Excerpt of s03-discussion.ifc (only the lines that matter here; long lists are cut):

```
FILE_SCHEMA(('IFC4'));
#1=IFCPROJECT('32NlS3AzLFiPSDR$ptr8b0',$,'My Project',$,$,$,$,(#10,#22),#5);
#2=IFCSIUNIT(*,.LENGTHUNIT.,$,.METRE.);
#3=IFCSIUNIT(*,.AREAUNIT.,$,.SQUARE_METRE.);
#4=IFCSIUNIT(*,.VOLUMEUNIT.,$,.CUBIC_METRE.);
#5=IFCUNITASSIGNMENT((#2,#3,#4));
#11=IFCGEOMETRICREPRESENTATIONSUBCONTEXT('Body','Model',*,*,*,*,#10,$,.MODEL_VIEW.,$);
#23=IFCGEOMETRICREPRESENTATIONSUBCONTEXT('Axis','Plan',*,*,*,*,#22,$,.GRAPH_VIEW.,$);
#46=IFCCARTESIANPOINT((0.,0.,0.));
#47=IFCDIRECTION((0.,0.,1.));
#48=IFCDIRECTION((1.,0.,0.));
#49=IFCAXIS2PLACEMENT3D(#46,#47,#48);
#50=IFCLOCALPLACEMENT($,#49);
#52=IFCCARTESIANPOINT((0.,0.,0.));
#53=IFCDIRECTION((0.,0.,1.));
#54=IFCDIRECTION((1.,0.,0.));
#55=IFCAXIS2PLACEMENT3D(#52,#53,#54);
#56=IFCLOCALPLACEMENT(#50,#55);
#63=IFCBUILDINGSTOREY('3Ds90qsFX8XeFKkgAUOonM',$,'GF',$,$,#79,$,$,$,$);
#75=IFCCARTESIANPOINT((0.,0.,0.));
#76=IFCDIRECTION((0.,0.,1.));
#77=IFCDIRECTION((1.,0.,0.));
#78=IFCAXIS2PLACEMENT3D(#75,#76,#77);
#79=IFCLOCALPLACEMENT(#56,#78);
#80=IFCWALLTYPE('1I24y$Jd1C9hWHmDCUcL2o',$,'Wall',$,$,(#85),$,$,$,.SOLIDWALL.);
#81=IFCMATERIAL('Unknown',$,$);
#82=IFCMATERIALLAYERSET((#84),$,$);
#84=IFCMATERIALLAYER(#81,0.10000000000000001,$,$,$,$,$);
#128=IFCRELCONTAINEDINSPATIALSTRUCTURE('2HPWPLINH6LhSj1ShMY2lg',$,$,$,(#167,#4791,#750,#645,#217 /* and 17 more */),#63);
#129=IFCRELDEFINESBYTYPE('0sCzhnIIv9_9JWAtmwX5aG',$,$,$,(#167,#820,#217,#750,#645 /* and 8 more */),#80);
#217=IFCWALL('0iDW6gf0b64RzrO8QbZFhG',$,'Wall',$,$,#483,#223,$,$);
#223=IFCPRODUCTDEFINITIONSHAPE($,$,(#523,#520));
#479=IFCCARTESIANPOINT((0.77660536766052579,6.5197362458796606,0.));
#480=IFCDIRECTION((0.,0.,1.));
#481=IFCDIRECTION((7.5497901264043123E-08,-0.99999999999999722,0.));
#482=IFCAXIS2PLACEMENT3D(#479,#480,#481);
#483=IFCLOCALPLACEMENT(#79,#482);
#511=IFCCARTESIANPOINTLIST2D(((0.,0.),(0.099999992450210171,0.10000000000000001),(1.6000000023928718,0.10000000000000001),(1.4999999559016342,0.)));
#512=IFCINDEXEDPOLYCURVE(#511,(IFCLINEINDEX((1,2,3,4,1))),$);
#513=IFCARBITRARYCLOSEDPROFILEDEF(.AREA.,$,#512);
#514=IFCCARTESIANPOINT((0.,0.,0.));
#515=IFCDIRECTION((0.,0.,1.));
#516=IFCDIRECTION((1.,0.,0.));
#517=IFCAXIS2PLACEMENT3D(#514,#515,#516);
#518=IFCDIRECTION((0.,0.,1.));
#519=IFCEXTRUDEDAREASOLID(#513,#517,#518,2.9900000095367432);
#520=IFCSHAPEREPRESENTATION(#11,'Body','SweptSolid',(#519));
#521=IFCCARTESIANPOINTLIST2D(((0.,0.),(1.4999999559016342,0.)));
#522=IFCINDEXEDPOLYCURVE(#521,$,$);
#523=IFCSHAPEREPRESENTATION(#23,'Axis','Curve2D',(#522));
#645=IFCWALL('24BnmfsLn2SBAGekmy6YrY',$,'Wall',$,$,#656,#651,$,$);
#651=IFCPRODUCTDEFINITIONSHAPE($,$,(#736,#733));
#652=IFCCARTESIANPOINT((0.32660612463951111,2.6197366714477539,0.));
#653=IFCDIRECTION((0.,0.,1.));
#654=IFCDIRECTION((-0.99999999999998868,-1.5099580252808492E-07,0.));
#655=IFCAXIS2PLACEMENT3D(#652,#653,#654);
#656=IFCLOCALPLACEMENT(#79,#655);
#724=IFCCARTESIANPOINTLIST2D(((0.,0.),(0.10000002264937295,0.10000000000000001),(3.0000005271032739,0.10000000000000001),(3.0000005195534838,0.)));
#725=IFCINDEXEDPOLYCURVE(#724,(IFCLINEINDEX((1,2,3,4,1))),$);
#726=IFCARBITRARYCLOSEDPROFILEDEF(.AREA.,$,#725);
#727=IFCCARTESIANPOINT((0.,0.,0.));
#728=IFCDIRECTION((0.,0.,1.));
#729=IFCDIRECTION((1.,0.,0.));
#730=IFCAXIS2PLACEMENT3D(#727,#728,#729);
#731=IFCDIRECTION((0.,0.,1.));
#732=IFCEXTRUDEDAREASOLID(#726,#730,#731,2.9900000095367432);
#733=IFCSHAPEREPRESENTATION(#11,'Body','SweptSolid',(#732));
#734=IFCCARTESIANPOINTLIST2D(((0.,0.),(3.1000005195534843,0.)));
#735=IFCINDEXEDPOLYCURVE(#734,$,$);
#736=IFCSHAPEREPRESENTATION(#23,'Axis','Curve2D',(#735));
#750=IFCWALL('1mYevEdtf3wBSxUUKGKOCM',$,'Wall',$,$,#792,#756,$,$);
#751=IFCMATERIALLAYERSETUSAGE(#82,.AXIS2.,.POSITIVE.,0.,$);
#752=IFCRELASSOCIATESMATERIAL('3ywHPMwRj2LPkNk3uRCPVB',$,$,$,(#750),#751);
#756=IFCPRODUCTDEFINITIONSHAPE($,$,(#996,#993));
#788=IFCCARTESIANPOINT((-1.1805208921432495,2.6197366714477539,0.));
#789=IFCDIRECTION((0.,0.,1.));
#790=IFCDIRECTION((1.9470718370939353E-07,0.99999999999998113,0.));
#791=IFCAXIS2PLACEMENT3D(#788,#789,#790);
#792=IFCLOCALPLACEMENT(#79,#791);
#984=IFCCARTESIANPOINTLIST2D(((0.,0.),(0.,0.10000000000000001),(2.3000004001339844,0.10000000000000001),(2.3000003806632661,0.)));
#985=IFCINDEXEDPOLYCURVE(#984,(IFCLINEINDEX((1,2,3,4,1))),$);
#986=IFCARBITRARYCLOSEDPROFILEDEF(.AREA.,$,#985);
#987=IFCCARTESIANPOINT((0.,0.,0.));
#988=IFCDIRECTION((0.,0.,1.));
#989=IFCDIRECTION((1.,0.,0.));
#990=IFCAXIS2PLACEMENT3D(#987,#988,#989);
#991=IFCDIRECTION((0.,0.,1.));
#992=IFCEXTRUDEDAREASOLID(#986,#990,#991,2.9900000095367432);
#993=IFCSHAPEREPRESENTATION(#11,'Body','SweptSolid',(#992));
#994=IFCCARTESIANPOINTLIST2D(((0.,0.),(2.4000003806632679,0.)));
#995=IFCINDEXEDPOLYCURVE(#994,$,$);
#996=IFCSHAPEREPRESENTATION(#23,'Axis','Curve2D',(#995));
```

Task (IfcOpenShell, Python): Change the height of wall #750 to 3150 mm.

```python
import ifcopenshell
import ifcopenshell.geom
import ifcopenshell.util.representation
import ifcopenshell.util.shape
import ifcopenshell.util.unit

model = ifcopenshell.open("s03-discussion.ifc")
unit_scale = ifcopenshell.util.unit.calculate_unit_scale(model)
settings = ifcopenshell.geom.settings()


def volume(element):
    """Net volume in cubic metres, openings subtracted."""
    shape = ifcopenshell.geom.create_shape(settings, element)
    return ifcopenshell.util.shape.get_volume(shape.geometry)


wall = model.by_id(750)
before = volume(wall)

body = ifcopenshell.util.representation.get_representation(wall, "Model", "Body")
solid = body.Items[0]
old_height = solid.Depth
solid.Depth = 3.15 / unit_scale
after = volume(wall)

print(f"height {old_height:g} -> {solid.Depth:g}, volume {before:.3f} -> {after:.3f} m3")

model.write("s03-discussion-out.ifc")
```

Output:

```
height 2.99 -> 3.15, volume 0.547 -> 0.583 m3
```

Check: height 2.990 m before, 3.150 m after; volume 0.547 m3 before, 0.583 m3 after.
